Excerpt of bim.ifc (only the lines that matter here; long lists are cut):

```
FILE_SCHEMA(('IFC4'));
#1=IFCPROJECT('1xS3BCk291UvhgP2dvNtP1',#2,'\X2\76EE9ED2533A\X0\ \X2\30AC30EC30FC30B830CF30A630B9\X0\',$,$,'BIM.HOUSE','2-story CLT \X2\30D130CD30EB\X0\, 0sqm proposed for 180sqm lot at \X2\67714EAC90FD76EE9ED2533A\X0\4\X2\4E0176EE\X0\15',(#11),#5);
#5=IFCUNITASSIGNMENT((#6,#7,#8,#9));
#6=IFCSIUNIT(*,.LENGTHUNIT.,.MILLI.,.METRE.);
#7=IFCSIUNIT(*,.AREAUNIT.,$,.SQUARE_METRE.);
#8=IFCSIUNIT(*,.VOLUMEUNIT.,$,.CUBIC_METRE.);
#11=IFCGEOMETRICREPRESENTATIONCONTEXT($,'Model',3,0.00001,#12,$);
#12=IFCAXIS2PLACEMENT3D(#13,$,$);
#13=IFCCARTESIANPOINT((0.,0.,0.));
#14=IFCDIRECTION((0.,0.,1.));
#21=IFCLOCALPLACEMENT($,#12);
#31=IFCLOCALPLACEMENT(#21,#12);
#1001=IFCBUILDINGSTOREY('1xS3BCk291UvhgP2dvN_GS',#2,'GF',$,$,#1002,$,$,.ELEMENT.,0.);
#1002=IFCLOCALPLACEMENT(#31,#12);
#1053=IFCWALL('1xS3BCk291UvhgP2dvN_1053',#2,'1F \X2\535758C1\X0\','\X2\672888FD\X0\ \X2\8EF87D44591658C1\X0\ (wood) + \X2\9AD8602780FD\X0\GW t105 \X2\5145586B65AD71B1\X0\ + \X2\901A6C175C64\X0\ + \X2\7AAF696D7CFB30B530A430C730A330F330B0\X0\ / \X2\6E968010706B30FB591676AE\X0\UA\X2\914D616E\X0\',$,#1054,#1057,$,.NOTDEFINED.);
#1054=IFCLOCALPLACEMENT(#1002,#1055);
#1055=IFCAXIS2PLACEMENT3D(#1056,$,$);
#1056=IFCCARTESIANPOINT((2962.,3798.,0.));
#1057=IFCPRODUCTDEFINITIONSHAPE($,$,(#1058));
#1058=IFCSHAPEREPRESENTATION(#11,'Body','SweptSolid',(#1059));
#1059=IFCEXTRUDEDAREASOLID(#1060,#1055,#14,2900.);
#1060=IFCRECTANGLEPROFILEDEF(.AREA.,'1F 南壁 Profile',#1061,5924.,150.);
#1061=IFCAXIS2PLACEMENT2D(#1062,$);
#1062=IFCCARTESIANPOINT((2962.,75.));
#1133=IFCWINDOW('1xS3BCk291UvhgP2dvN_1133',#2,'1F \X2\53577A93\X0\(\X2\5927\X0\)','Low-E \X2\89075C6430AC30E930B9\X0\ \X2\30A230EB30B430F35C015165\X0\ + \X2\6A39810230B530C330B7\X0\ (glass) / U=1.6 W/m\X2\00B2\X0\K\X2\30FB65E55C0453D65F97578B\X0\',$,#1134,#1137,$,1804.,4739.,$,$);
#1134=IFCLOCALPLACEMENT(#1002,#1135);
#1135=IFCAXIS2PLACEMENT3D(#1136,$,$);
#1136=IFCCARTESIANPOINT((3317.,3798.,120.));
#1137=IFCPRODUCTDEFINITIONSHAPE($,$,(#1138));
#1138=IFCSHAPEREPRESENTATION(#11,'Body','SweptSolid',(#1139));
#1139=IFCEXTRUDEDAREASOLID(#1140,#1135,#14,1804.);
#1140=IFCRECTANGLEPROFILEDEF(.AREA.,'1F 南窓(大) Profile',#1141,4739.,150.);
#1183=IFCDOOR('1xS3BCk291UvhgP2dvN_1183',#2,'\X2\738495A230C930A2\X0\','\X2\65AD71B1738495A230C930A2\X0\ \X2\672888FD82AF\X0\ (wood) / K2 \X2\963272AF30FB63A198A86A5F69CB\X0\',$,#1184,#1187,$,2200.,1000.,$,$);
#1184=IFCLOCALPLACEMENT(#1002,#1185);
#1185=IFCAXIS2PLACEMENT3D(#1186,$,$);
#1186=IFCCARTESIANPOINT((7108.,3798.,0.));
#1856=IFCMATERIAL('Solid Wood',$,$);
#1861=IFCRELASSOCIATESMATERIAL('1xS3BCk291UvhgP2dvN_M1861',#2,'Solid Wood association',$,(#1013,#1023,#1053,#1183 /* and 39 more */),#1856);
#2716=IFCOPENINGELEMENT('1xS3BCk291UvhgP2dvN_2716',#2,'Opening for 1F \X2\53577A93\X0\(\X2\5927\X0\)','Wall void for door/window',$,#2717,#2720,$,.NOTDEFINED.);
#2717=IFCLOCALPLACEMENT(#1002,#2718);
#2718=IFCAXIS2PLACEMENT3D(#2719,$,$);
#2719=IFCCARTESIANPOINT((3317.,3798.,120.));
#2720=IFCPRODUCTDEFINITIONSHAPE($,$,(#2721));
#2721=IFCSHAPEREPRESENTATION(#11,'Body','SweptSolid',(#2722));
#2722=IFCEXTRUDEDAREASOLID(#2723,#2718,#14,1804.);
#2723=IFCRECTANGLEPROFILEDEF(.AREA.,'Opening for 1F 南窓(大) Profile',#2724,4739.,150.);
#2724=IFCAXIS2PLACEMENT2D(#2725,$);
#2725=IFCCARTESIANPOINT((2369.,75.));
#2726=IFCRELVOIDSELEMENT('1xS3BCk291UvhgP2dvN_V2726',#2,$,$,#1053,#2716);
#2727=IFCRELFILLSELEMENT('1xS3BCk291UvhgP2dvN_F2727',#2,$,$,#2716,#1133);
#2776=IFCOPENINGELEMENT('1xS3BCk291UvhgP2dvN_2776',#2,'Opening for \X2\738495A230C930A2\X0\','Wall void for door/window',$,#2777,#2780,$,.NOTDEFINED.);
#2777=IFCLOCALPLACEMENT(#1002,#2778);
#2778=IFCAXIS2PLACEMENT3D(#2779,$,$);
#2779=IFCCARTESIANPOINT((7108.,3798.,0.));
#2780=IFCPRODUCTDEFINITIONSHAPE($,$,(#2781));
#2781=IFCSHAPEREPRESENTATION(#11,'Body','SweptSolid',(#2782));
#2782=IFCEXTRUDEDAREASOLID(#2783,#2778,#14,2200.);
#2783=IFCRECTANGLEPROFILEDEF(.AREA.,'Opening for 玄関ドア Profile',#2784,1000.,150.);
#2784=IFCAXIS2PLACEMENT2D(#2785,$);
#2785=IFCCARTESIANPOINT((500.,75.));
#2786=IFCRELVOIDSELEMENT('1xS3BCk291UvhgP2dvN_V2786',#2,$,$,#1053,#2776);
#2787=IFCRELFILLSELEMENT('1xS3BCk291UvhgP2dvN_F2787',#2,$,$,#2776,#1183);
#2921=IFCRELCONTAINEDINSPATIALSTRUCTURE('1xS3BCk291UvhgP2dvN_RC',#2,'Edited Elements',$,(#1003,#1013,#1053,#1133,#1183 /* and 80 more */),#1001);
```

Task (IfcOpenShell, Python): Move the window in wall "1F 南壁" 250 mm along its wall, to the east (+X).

```python
import ifcopenshell
import ifcopenshell.api.geometry
import ifcopenshell.util.placement
import ifcopenshell.util.unit

model = ifcopenshell.open("bim.ifc")
unit_scale = ifcopenshell.util.unit.calculate_unit_scale(model)

window = model.by_id(1133)
opening = window.FillsVoids[0].RelatingOpeningElement
wall = opening.VoidsElements[0].RelatingBuildingElement

wall_matrix = ifcopenshell.util.placement.get_local_placement(wall.ObjectPlacement)
shift = wall_matrix[:3, 0] * 0.25 / unit_scale
before = ifcopenshell.util.placement.get_local_placement(window.ObjectPlacement)[:3, 3].copy()

# The window is not placed relative to its opening, so move both.
for product in (opening, window):
    matrix = ifcopenshell.util.placement.get_local_placement(product.ObjectPlacement)
    matrix[:3, 3] += shift
    ifcopenshell.api.geometry.edit_object_placement(model, product=product, matrix=matrix, is_si=False)

after = ifcopenshell.util.placement.get_local_placement(window.ObjectPlacement)[:3, 3]
print("window moved by", (after - before).round(3) + 0.0)

model.write("bim-out.ifc")
```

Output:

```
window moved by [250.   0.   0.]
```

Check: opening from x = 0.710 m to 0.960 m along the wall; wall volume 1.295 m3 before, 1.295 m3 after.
